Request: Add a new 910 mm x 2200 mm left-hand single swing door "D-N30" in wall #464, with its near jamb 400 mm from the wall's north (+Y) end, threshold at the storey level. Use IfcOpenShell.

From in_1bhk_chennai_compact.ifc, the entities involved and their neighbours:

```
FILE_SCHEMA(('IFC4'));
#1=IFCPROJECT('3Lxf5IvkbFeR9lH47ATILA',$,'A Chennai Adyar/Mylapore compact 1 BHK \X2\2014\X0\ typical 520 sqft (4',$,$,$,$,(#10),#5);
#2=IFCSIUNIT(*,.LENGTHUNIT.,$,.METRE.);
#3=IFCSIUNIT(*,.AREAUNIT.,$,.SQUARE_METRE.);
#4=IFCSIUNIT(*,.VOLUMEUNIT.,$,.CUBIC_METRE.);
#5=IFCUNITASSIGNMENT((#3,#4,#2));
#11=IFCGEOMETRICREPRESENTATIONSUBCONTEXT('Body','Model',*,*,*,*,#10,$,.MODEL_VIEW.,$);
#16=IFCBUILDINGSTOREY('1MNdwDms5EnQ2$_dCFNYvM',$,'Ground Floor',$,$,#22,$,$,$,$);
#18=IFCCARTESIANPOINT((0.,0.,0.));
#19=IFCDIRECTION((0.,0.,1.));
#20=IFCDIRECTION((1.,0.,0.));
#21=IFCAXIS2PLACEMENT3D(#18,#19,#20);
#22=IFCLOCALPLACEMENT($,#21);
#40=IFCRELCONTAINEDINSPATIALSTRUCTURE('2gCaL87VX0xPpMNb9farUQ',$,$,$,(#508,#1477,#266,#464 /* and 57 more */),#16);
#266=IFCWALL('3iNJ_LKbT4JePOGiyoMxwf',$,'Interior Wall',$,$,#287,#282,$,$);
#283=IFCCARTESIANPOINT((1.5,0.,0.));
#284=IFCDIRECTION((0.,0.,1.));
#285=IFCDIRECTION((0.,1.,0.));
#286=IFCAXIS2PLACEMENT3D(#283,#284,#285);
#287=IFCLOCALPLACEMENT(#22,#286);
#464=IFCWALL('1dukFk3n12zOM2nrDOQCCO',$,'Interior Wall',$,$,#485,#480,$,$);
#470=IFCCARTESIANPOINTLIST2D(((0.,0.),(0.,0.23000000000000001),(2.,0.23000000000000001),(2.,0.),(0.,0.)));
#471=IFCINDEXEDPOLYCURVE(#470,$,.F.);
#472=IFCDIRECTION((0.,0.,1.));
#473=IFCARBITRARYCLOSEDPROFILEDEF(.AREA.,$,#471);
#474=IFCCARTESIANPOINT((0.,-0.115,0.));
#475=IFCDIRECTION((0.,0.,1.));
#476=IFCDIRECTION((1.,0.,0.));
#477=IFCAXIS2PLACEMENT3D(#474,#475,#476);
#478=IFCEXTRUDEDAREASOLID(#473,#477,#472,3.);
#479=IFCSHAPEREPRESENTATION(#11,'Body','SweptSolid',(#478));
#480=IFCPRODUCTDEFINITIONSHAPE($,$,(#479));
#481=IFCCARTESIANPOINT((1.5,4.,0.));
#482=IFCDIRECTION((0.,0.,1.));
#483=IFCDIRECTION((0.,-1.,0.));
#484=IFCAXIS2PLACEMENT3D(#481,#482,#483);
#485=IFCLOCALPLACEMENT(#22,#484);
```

```python
import numpy as np
import ifcopenshell
import ifcopenshell.api.feature
import ifcopenshell.api.geometry
import ifcopenshell.api.root
import ifcopenshell.api.spatial
import ifcopenshell.geom
import ifcopenshell.util.element
import ifcopenshell.util.placement
import ifcopenshell.util.representation
import ifcopenshell.util.shape
import ifcopenshell.util.unit

model = ifcopenshell.open("in_1bhk_chennai_compact.ifc")
unit_scale = ifcopenshell.util.unit.calculate_unit_scale(model)
settings = ifcopenshell.geom.settings()


def volume(element):
    """Net volume in cubic metres, openings subtracted."""
    shape = ifcopenshell.geom.create_shape(settings, element)
    return ifcopenshell.util.shape.get_volume(shape.geometry)


wall = model.by_guid("1dukFk3n12zOM2nrDOQCCO")
storey = ifcopenshell.util.element.get_container(wall, ifc_class="IfcBuildingStorey")
context = ifcopenshell.util.representation.get_context(model, "Model", "Body", "MODEL_VIEW")
before = volume(wall)

width, height, from_end, sill = 0.91, 2.2, 0.4, 0.0  # metres

# The wall runs along its own X axis, and the end named is its -X end.
wall_shape = ifcopenshell.geom.create_shape(settings, wall)
x, y, z = ifcopenshell.util.shape.get_vertices(wall_shape.geometry).T
start = x.min() + from_end
face, thickness = float(y.min()), float(y.max() - y.min())
wall_matrix = ifcopenshell.util.placement.get_local_placement(wall.ObjectPlacement)
level = ifcopenshell.util.placement.get_local_placement(storey.ObjectPlacement)[2, 3]


def in_wall(x, y):
    """Placement at x, y metres in the wall's axes, at sill height."""
    matrix = wall_matrix.copy()
    matrix[:, 3] = wall_matrix @ np.array([x / unit_scale, y / unit_scale, 0.0, 1.0])
    matrix[2, 3] = level + sill / unit_scale
    return matrix


# Opening: a box that overshoots both wall faces by 50 mm.
opening = ifcopenshell.api.root.create_entity(model, ifc_class="IfcOpeningElement", predefined_type="OPENING")
box = ifcopenshell.api.geometry.add_wall_representation(
    model, context=context, length=width, height=height, thickness=thickness + 0.1
)
ifcopenshell.api.geometry.assign_representation(model, product=opening, representation=box)
ifcopenshell.api.geometry.edit_object_placement(model, product=opening, matrix=in_wall(start, face - 0.05), is_si=False)
ifcopenshell.api.feature.add_feature(model, feature=opening, element=wall)

door = ifcopenshell.api.root.create_entity(model, ifc_class="IfcDoor", name="D-N30", predefined_type="DOOR")
door.OverallWidth, door.OverallHeight = width / unit_scale, height / unit_scale
door.OperationType = "SINGLE_SWING_LEFT"
body = ifcopenshell.api.geometry.add_door_representation(
    model,
    context=context,
    overall_width=door.OverallWidth,
    overall_height=door.OverallHeight,
    operation_type="SINGLE_SWING_LEFT",
    lining_properties={"LiningDepth": thickness / unit_scale, "ThresholdDepth": thickness / unit_scale},
)
ifcopenshell.api.geometry.assign_representation(model, product=door, representation=body)
ifcopenshell.api.spatial.assign_container(model, products=[door], relating_structure=storey)
ifcopenshell.api.feature.add_filling(model, opening=opening, element=door)

# The lining spans the wall, so the door starts at the wall face.
ifcopenshell.api.geometry.edit_object_placement(model, product=door, matrix=in_wall(start, face), is_si=False)

after = volume(wall)

print(f"wall volume {before:.3f} -> {after:.3f} m3")

model.write("in_1bhk_chennai_compact_updated.ifc")
```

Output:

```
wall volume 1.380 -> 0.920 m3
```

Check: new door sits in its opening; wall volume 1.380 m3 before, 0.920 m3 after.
